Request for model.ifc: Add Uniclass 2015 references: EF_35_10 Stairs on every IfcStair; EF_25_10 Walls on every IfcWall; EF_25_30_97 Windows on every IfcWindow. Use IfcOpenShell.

First a look at what the model holds.

```python
import ifcopenshell

model = ifcopenshell.open("model.ifc")
print(model.schema)
print("classifications:", [c.Name for c in model.by_type("IfcClassification")])
for ifc_class in ("IfcDoor", "IfcRoof", "IfcStair", "IfcWall", "IfcWindow"):
    print(ifc_class, len(model.by_type(ifc_class)))
```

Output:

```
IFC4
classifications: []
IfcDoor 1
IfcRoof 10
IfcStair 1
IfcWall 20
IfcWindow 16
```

```python
import ifcopenshell
import ifcopenshell.api.classification

model = ifcopenshell.open("model.ifc")

system = ifcopenshell.api.classification.add_classification(model, classification="Uniclass 2015")

codes = {
    "IfcStair": ("EF_35_10", "Stairs"),
    "IfcWall": ("EF_25_10", "Walls"),
    "IfcWindow": ("EF_25_30_97", "Windows"),
}
for ifc_class, (code, name) in codes.items():
    products = model.by_type(ifc_class)
    ifcopenshell.api.classification.add_reference(
        model, products=products, classification=system, identification=code, name=name
    )
    print(code, len(products))

model.write("model_updated.ifc")
```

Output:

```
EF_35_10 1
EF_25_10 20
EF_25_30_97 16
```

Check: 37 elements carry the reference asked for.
